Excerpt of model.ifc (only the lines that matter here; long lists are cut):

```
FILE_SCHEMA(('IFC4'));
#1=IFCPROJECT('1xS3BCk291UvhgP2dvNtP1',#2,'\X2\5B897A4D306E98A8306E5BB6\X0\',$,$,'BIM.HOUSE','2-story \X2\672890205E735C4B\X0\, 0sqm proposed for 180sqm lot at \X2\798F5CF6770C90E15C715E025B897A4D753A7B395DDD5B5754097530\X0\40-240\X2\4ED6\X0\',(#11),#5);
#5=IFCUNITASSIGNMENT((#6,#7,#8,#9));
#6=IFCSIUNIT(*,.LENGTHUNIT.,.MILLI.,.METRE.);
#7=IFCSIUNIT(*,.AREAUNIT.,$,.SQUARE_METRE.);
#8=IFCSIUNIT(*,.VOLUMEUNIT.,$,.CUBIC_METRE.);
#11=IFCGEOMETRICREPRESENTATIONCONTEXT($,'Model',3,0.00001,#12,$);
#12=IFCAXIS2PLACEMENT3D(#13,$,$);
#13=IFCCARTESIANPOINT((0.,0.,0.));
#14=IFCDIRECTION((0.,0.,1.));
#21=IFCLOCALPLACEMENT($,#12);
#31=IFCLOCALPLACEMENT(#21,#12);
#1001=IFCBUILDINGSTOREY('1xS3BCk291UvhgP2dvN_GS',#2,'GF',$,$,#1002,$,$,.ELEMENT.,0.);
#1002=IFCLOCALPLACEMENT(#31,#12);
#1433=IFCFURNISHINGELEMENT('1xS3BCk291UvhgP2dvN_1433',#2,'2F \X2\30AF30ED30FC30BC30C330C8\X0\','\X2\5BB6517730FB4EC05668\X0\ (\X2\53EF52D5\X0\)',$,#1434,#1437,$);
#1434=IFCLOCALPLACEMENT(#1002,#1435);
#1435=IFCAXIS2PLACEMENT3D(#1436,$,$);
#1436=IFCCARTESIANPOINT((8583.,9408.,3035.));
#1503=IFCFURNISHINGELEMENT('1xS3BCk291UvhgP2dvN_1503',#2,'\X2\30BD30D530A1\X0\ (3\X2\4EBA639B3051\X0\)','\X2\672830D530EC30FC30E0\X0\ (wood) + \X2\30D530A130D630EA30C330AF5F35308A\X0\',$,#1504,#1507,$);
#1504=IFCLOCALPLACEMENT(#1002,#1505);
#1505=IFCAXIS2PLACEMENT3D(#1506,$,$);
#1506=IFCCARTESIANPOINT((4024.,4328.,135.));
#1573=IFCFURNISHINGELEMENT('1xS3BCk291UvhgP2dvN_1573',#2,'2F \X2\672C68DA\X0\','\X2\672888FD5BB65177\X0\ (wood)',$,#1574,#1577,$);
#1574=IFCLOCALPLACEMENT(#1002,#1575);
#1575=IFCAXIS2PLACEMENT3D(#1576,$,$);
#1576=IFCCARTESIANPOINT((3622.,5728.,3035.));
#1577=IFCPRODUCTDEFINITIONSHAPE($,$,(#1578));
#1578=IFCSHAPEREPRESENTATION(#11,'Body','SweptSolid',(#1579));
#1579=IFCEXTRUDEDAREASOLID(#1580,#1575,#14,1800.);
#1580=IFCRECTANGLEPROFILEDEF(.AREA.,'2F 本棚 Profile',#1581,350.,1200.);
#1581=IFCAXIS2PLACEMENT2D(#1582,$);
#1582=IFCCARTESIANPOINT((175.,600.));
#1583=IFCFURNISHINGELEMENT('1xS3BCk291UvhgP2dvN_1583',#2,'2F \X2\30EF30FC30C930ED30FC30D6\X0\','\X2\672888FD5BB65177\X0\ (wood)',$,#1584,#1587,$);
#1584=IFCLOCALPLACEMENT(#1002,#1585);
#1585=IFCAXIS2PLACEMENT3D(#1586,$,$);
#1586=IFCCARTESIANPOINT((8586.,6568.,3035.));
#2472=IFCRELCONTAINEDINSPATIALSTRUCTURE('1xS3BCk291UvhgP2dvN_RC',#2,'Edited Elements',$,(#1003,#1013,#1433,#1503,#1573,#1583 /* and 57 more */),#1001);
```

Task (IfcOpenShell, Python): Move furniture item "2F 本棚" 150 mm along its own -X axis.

```python
import ifcopenshell
import ifcopenshell.api.geometry
import ifcopenshell.util.placement
import ifcopenshell.util.unit

model = ifcopenshell.open("model.ifc")
unit_scale = ifcopenshell.util.unit.calculate_unit_scale(model)

item = model.by_guid("1xS3BCk291UvhgP2dvN_1573")
matrix = ifcopenshell.util.placement.get_local_placement(item.ObjectPlacement)
matrix[:3, 3] -= matrix[:3, 0] * 0.15 / unit_scale
ifcopenshell.api.geometry.edit_object_placement(model, product=item, matrix=matrix, is_si=False)

print(ifcopenshell.util.placement.get_local_placement(item.ObjectPlacement).round(3) + 0.0)

model.write("model_v2.ifc")
```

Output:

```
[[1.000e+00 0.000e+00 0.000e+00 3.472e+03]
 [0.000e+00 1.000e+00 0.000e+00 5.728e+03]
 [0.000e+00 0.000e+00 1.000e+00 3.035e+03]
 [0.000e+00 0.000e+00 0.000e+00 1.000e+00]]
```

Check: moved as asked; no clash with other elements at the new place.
